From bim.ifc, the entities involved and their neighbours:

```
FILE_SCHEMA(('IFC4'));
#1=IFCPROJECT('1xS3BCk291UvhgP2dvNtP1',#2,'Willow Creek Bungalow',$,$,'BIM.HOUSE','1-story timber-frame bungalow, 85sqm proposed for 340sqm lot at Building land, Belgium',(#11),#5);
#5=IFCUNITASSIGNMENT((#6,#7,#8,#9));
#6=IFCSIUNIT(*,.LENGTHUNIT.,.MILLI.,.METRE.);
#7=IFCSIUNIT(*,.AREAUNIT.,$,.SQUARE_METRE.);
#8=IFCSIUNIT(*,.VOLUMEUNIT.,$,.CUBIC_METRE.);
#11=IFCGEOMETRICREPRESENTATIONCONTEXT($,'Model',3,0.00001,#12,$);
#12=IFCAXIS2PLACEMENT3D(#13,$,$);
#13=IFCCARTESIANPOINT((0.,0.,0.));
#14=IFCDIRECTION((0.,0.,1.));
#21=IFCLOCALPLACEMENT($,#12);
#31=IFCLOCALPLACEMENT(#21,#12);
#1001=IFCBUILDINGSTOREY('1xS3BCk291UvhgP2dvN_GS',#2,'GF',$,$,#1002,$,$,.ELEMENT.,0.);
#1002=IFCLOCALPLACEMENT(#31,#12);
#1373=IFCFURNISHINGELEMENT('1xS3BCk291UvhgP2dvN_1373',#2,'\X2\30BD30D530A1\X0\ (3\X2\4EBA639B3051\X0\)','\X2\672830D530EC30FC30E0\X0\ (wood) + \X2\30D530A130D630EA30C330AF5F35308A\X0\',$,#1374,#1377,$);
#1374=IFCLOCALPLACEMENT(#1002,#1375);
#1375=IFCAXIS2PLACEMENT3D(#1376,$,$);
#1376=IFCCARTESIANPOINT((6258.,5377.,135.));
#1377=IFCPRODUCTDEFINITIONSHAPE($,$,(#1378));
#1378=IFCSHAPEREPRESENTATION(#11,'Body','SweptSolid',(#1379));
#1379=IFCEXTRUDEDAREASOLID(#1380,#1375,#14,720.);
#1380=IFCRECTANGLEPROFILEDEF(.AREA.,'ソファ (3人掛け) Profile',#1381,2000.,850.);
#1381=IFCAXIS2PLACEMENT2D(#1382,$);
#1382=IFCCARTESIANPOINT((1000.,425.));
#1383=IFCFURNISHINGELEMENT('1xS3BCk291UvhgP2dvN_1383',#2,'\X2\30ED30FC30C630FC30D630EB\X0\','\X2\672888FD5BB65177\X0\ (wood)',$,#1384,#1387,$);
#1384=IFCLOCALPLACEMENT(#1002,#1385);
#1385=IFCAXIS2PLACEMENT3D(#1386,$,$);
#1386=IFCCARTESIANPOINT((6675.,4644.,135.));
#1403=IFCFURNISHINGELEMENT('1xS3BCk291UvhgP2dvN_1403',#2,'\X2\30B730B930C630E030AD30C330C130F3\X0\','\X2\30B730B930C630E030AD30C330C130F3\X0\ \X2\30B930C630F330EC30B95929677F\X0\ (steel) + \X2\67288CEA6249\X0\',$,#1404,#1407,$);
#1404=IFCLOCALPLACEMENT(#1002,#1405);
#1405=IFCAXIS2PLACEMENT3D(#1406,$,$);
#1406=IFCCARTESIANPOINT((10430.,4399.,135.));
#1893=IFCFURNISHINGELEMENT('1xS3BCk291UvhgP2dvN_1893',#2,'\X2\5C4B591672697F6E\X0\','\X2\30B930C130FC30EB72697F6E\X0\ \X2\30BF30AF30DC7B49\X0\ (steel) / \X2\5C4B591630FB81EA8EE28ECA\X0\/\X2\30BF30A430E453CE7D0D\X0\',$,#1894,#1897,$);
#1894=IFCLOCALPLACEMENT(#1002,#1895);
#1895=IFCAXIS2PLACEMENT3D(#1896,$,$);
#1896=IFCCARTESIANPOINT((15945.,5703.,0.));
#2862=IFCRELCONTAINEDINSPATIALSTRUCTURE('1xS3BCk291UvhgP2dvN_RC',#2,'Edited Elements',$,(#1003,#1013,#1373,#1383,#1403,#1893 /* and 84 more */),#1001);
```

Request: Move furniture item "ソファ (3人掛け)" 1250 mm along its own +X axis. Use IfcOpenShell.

```python
import ifcopenshell
import ifcopenshell.api.geometry
import ifcopenshell.util.placement

model = ifcopenshell.open("bim.ifc")

item = model.by_id(1373)
matrix = ifcopenshell.util.placement.get_local_placement(item.ObjectPlacement)
matrix[:3, 3] += matrix[:3, 0] * 1250.0
ifcopenshell.api.geometry.edit_object_placement(model, product=item, matrix=matrix, is_si=False)

print(ifcopenshell.util.placement.get_local_placement(item.ObjectPlacement).round(3) + 0.0)

model.write("bim_rev.ifc")
```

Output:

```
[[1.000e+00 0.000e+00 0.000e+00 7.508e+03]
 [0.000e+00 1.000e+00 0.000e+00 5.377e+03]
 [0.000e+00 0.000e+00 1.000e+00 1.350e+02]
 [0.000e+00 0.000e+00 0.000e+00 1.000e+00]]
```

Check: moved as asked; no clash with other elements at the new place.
